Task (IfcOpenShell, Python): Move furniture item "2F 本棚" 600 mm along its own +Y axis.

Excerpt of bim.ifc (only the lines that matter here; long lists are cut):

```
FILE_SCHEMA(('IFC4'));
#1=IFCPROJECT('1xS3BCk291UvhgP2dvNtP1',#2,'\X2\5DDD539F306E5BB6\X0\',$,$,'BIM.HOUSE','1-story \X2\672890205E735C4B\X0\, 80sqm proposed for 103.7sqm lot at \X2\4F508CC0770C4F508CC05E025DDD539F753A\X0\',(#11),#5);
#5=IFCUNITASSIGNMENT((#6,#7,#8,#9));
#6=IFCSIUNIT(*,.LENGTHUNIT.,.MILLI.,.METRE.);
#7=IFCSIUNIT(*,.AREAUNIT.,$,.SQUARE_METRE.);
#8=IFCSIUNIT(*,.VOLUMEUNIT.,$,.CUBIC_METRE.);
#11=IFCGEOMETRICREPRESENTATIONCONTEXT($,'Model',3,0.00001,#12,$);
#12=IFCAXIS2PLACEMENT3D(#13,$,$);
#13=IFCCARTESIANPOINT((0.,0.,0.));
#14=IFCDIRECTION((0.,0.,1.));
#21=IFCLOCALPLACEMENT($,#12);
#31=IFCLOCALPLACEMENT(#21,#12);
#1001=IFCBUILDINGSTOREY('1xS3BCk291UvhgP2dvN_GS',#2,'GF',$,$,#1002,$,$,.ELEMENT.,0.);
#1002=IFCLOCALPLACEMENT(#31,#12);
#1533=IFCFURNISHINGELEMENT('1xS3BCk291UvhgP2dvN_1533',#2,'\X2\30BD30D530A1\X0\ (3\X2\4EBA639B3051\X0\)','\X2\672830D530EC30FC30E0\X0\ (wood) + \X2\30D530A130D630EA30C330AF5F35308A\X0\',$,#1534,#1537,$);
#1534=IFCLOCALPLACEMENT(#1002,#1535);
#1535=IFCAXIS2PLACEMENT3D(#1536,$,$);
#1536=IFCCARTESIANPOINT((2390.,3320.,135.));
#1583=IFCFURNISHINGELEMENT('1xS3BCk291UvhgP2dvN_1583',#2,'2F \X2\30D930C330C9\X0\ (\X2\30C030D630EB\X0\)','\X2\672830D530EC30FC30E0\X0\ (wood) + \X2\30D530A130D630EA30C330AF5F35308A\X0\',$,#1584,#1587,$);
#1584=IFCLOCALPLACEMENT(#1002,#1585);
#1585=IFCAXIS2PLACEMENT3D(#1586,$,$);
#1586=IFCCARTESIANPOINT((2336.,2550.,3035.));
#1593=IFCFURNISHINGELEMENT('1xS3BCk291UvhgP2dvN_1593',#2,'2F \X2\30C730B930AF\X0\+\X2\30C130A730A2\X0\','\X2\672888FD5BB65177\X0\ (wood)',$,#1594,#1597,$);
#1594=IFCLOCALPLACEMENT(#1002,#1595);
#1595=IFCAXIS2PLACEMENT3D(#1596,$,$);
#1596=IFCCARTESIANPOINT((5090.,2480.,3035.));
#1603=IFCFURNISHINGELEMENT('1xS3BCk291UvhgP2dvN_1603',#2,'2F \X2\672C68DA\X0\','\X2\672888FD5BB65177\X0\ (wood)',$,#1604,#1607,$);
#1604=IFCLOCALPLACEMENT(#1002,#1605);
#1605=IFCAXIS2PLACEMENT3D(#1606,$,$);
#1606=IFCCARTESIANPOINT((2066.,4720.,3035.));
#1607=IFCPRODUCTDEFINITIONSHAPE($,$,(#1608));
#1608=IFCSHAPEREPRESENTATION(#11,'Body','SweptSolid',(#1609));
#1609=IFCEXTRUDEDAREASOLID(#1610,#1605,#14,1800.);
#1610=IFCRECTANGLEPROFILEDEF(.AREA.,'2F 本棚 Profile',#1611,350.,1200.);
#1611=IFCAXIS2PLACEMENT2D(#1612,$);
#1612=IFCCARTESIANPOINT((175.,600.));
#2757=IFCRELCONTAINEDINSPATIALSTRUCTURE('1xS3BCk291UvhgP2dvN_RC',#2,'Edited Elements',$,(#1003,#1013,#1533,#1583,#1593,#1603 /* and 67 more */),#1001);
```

```python
import ifcopenshell
import ifcopenshell.api.geometry
import ifcopenshell.util.placement

model = ifcopenshell.open("bim.ifc")

item = model.by_guid("1xS3BCk291UvhgP2dvN_1603")
matrix = ifcopenshell.util.placement.get_local_placement(item.ObjectPlacement)
matrix[:3, 3] += matrix[:3, 1] * 600.0
ifcopenshell.api.geometry.edit_object_placement(model, product=item, matrix=matrix, is_si=False)

print(ifcopenshell.util.placement.get_local_placement(item.ObjectPlacement).round(3) + 0.0)

model.write("bim_updated.ifc")
```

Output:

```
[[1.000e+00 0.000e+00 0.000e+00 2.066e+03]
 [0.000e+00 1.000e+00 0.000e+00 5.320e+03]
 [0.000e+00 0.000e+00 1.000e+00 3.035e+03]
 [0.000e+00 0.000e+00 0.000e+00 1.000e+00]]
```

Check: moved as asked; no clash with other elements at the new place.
